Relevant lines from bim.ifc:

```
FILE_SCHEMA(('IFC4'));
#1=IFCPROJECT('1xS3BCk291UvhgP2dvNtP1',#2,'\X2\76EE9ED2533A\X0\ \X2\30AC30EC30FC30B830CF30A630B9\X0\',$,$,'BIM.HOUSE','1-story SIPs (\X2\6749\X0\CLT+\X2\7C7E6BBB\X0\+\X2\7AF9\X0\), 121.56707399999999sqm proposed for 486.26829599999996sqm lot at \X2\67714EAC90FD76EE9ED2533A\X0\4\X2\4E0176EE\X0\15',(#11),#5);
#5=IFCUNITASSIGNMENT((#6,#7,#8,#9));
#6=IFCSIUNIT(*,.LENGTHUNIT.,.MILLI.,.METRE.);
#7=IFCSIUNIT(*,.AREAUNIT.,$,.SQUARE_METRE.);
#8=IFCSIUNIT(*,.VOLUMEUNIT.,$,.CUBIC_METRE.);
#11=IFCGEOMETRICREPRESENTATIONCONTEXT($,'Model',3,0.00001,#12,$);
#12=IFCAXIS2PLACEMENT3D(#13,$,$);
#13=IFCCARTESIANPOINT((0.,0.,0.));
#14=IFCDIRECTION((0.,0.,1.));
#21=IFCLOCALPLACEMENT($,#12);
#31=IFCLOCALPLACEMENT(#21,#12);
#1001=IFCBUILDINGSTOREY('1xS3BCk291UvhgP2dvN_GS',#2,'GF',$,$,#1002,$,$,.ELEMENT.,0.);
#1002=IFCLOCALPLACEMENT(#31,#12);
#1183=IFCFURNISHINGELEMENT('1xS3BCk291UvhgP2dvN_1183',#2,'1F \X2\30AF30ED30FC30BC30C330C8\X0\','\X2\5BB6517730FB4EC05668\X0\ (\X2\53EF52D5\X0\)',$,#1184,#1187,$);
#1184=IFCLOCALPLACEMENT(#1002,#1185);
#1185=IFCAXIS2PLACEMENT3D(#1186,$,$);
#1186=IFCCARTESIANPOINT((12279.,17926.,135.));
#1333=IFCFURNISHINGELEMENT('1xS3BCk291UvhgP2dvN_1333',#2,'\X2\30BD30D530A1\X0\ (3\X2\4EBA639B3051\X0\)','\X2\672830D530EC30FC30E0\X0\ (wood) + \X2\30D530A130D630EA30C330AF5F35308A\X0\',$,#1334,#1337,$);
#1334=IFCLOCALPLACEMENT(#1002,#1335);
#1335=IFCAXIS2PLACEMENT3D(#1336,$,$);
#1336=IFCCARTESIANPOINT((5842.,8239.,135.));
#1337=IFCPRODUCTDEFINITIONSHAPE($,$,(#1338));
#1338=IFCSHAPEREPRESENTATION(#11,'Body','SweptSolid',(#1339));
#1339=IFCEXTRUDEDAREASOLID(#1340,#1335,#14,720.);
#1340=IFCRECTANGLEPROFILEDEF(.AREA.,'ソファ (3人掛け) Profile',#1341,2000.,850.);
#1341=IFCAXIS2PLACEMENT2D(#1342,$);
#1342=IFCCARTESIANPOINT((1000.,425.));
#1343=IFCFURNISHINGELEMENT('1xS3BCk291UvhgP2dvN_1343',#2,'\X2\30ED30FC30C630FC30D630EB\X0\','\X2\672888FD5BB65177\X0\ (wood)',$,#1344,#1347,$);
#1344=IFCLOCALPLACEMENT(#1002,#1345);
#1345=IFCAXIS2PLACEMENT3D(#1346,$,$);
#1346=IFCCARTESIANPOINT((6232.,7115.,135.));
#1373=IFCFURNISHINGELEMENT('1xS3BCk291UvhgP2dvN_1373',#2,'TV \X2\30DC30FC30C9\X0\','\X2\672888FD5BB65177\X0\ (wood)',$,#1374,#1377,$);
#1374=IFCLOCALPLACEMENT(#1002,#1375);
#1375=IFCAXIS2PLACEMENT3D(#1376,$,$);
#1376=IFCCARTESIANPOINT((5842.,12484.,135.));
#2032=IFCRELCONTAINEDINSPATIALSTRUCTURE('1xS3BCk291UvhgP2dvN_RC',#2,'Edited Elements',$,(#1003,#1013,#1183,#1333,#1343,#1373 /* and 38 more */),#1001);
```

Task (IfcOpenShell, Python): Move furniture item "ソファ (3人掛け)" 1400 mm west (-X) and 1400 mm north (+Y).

```python
import ifcopenshell
import ifcopenshell.api.geometry
import ifcopenshell.util.placement
import ifcopenshell.util.unit

model = ifcopenshell.open("bim.ifc")
unit_scale = ifcopenshell.util.unit.calculate_unit_scale(model)

item = model.by_guid("1xS3BCk291UvhgP2dvN_1333")
matrix = ifcopenshell.util.placement.get_local_placement(item.ObjectPlacement)
matrix[0, 3] -= 1.4 / unit_scale
matrix[1, 3] += 1.4 / unit_scale
ifcopenshell.api.geometry.edit_object_placement(model, product=item, matrix=matrix, is_si=False)

print(ifcopenshell.util.placement.get_local_placement(item.ObjectPlacement).round(3) + 0.0)

model.write("bim_updated.ifc")
```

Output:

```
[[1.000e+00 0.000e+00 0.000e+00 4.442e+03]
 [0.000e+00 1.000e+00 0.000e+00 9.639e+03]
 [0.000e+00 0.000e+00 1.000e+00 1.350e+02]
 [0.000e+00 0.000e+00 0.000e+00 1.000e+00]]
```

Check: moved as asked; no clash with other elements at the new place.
